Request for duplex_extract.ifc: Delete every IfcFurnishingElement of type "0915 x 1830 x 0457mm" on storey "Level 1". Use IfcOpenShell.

First a look at what the model holds.

```python
import ifcopenshell
import ifcopenshell.util.element

model = ifcopenshell.open("duplex_extract.ifc")
print(model.schema)
storey = next(s for s in model.by_type("IfcBuildingStorey") if s.Name == "Level 1")
furniture = [e for e in ifcopenshell.util.element.get_decomposition(storey) if e.is_a("IfcFurnishingElement")]
seen = {}
for e in furniture:
    element_type = ifcopenshell.util.element.get_type(e)
    name = element_type.Name if element_type not in (None, e) else None
    seen[name] = seen.get(name, 0) + 1
for name, count in sorted(seen.items(), key=str):
    print(count, "x", name)
```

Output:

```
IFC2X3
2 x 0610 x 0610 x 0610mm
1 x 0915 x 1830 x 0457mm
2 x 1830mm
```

```python
import ifcopenshell
import ifcopenshell.api.root
import ifcopenshell.util.element

model = ifcopenshell.open("duplex_extract.ifc")

storey = next(s for s in model.by_type("IfcBuildingStorey") if s.Name == "Level 1")
furniture = [e for e in ifcopenshell.util.element.get_decomposition(storey) if e.is_a("IfcFurnishingElement")]
targets = [e for e in furniture if (t := ifcopenshell.util.element.get_type(e)) not in (None, e) and t.Name == "0915 x 1830 x 0457mm"]

for e in targets:
    ifcopenshell.api.root.remove_product(model, product=e)
print(len(targets), "removed")

model.write("duplex_extract_v2.ifc")
```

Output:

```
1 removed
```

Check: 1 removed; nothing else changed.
